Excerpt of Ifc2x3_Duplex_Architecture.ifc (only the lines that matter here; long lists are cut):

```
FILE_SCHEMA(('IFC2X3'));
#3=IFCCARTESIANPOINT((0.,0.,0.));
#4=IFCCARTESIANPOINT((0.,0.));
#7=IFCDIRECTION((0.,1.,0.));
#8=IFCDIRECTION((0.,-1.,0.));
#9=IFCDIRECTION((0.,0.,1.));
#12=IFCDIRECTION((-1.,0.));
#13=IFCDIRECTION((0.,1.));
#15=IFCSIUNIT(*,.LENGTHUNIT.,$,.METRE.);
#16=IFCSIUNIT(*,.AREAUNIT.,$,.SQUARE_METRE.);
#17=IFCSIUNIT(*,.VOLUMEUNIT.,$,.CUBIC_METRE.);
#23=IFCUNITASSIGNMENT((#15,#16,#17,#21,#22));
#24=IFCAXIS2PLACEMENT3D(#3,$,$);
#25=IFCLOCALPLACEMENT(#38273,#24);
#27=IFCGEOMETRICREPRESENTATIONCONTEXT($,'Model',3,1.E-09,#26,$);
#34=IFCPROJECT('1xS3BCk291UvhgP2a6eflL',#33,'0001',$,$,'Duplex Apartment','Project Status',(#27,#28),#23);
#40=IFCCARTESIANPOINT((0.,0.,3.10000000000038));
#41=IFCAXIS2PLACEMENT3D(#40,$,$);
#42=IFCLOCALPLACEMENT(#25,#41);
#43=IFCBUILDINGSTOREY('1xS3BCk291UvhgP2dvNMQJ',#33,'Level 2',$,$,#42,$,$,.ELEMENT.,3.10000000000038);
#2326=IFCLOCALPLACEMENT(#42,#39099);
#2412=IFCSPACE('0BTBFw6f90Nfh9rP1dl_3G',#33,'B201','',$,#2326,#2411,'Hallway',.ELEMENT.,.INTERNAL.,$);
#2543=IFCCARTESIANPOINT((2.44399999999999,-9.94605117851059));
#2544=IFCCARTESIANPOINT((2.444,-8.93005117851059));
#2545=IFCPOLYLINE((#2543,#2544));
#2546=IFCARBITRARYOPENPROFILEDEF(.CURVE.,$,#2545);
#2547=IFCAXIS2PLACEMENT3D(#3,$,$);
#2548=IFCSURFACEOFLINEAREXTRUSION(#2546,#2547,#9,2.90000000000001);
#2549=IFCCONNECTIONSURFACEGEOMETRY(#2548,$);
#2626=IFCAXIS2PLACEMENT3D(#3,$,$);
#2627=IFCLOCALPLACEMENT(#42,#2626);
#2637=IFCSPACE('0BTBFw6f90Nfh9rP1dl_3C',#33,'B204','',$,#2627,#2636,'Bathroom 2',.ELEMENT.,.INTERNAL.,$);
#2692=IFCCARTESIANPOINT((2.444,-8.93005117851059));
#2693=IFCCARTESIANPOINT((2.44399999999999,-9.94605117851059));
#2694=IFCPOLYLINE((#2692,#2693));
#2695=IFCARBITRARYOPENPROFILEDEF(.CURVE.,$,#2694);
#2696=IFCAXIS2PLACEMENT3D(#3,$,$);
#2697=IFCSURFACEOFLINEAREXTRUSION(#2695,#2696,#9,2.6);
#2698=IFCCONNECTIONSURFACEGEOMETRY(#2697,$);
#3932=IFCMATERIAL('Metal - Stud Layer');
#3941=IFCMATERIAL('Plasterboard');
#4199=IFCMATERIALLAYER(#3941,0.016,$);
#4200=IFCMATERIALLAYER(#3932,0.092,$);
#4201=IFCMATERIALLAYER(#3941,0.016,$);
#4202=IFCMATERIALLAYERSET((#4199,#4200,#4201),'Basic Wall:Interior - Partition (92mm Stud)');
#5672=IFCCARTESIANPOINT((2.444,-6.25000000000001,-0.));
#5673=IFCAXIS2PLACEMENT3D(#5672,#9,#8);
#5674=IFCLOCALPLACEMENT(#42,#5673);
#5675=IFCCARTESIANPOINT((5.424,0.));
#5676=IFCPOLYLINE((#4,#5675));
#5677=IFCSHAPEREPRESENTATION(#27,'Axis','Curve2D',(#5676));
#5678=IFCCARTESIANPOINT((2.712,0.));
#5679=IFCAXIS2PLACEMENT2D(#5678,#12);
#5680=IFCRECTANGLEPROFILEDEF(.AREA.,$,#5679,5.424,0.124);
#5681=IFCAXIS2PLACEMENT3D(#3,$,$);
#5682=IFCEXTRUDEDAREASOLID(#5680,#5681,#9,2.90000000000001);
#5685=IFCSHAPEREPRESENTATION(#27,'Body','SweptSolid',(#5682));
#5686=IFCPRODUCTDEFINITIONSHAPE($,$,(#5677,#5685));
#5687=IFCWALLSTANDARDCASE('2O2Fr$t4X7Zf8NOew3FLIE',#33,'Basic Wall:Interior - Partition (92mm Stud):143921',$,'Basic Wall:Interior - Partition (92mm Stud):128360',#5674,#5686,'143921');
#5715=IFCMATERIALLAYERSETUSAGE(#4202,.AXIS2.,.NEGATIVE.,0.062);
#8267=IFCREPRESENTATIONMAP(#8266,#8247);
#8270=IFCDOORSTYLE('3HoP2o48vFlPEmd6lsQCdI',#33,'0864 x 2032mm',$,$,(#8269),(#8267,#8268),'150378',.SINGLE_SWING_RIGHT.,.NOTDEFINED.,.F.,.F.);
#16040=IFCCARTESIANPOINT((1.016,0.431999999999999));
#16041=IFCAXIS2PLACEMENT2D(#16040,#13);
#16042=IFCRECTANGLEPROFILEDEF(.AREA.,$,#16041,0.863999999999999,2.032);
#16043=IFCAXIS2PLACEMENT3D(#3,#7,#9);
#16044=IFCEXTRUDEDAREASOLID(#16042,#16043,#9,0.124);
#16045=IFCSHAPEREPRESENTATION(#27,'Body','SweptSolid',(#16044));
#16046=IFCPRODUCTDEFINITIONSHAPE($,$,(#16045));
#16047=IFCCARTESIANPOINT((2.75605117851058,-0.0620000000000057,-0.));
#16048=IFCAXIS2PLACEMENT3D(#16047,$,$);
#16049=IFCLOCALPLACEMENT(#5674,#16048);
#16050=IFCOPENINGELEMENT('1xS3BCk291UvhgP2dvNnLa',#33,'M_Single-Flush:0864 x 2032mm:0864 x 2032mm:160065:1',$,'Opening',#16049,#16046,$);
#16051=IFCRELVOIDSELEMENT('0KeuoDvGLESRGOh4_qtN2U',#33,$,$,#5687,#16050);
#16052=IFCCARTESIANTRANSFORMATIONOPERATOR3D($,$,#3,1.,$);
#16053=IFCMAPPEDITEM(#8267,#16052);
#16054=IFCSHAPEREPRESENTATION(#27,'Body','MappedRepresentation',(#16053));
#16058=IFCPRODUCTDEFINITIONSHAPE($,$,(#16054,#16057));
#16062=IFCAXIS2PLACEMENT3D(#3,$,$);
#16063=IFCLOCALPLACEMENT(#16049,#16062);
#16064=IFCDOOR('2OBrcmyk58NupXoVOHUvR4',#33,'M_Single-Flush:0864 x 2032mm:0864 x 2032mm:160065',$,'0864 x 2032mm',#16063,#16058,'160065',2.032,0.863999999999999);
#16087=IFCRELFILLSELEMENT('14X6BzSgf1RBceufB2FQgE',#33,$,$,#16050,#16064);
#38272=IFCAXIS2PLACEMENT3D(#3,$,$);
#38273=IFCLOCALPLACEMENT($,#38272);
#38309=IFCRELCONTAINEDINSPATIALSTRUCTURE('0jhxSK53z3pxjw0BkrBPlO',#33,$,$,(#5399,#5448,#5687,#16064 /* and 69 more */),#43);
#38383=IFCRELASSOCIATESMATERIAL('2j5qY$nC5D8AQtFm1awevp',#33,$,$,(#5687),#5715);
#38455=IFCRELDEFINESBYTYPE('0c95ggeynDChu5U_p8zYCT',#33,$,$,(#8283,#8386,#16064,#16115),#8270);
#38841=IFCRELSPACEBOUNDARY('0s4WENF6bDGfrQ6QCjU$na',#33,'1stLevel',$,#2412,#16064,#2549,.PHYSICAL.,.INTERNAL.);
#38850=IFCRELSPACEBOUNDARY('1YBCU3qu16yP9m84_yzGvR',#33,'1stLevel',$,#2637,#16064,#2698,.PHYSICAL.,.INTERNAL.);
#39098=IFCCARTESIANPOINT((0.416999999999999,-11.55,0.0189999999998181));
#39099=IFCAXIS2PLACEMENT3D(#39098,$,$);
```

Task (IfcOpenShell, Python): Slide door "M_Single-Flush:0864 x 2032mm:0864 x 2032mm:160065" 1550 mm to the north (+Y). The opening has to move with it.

```python
import numpy as np
import ifcopenshell
import ifcopenshell.api.geometry
import ifcopenshell.util.placement
import ifcopenshell.util.unit

model = ifcopenshell.open("Ifc2x3_Duplex_Architecture.ifc")
unit_scale = ifcopenshell.util.unit.calculate_unit_scale(model)

door = model.by_guid("2OBrcmyk58NupXoVOHUvR4")
opening = door.FillsVoids[0].RelatingOpeningElement
wall = opening.VoidsElements[0].RelatingBuildingElement

wall_matrix = ifcopenshell.util.placement.get_local_placement(wall.ObjectPlacement)
shift = wall_matrix[:3, 0] * -1.55 / unit_scale
before = ifcopenshell.util.placement.get_local_placement(door.ObjectPlacement)[:3, 3].copy()

# The door is placed relative to its opening, so it follows when the opening moves.
matrix = ifcopenshell.util.placement.get_local_placement(opening.ObjectPlacement)
matrix[:3, 3] += shift
ifcopenshell.api.geometry.edit_object_placement(
    model, product=opening, matrix=matrix, is_si=False, should_transform_children=True
)

# Space boundary surfaces are stored in each space's coordinates; move them too.
for rel in door.ProvidesBoundaries:
    if not rel.ConnectionGeometry:
        continue
    surface = rel.ConnectionGeometry.SurfaceOnRelatingElement
    space_matrix = ifcopenshell.util.placement.get_local_placement(rel.RelatingSpace.ObjectPlacement)
    point = np.array(surface.Position.Location.Coordinates) + space_matrix[:3, :3].T @ shift
    surface.Position = model.createIfcAxis2Placement3D(
        model.createIfcCartesianPoint(point.tolist()), surface.Position.Axis, surface.Position.RefDirection
    )

after = ifcopenshell.util.placement.get_local_placement(door.ObjectPlacement)[:3, 3]
print("door moved by", (after - before).round(3) + 0.0)

model.write("Ifc2x3_Duplex_Architecture_edited.ifc")
```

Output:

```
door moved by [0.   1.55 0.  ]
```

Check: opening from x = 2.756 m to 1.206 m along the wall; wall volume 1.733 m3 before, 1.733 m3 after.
